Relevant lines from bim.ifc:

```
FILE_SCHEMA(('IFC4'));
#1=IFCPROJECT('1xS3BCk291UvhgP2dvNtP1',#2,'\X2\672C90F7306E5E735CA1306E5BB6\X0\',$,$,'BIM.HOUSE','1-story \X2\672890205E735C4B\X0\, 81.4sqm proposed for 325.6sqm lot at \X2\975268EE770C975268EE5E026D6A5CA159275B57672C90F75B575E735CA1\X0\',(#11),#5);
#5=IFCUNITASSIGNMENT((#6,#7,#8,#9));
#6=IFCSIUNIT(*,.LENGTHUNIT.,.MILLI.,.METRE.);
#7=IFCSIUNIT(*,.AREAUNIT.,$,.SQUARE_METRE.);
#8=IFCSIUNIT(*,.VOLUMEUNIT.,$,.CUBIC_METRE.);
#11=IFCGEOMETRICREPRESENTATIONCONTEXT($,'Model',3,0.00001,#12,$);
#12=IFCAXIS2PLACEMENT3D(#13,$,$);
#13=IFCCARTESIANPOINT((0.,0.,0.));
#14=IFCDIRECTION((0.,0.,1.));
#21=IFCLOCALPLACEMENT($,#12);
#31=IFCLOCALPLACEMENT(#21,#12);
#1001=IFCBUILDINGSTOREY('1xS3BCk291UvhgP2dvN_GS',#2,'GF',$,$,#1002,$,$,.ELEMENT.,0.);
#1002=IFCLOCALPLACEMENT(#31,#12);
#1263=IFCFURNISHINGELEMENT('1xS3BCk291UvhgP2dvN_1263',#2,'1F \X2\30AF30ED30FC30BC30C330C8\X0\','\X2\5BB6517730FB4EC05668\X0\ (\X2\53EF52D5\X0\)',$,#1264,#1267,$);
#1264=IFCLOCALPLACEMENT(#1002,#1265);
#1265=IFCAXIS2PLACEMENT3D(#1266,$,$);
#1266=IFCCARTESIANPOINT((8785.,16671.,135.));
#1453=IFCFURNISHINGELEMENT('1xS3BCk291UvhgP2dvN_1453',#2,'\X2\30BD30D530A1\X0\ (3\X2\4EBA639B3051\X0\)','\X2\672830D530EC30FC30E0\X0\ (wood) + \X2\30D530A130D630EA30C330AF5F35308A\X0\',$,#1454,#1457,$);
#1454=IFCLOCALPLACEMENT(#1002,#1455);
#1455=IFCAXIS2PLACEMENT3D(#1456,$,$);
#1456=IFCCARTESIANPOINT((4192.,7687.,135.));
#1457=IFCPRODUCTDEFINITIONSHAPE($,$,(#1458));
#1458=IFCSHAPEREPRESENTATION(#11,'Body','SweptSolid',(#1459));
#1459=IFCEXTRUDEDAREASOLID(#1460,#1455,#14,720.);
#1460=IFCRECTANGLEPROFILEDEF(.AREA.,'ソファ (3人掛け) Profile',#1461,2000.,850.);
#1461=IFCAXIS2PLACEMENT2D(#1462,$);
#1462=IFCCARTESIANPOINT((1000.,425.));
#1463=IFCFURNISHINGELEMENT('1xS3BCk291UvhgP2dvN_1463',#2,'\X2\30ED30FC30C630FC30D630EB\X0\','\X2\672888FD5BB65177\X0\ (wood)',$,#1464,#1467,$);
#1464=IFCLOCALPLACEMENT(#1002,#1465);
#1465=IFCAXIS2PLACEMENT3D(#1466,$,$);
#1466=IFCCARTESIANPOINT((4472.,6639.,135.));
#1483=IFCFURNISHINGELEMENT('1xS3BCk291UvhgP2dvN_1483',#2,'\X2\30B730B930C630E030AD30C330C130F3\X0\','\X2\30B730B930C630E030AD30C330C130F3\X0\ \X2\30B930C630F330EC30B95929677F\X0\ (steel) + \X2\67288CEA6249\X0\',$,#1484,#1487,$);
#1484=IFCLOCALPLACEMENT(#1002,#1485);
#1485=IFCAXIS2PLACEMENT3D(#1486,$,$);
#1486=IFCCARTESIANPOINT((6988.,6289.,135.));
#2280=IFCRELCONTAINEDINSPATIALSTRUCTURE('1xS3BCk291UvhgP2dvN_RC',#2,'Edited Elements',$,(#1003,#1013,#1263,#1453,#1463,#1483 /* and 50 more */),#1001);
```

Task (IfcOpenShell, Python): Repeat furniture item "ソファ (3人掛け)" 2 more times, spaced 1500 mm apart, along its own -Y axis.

```python
import ifcopenshell
import ifcopenshell.api.geometry
import ifcopenshell.api.root
import ifcopenshell.util.element
import ifcopenshell.util.placement
import ifcopenshell.util.unit

model = ifcopenshell.open("bim.ifc")
unit_scale = ifcopenshell.util.unit.calculate_unit_scale(model)


def reuse_history(source, copy):
    """copy_class also copies each property set's owner history, people and application; keep the originals."""
    for rel in copy.IsDefinedBy:
        if rel.is_a("IfcRelDefinesByProperties") and (history := rel.RelatingPropertyDefinition.OwnerHistory):
            rel.RelatingPropertyDefinition.OwnerHistory = source.OwnerHistory
            ifcopenshell.util.element.remove_deep2(model, history)


source = model.by_id(1453)
base = ifcopenshell.util.placement.get_local_placement(source.ObjectPlacement)
step = -base[:3, 1] * 1.5 / unit_scale

for i in range(1, 3):
    copy = ifcopenshell.api.root.copy_class(model, product=source)
    copy.Representation = ifcopenshell.util.element.copy_deep(
        model, source.Representation, exclude=["IfcGeometricRepresentationContext", "IfcRepresentationMap"]
    )
    reuse_history(source, copy)
    matrix = base.copy()
    matrix[:3, 3] += i * step
    print("added at", matrix[:3, 3].round(3) + 0.0)
    ifcopenshell.api.geometry.edit_object_placement(model, product=copy, matrix=matrix, is_si=False)

model.write("bim_edited.ifc")
```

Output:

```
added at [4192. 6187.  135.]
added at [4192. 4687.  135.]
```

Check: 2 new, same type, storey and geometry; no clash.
